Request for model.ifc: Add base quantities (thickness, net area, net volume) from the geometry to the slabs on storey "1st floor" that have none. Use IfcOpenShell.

First a look at what the model holds.

```python
import ifcopenshell
import ifcopenshell.util.element
import ifcopenshell.util.unit

model = ifcopenshell.open("model.ifc")
print(model.schema)
for unit_type in ("LENGTHUNIT", "AREAUNIT", "VOLUMEUNIT"):
    print(unit_type, ifcopenshell.util.unit.calculate_unit_scale(model, unit_type))
storey = next(s for s in model.by_type("IfcBuildingStorey") if s.Name == "1st floor")
slabs = [e for e in ifcopenshell.util.element.get_decomposition(storey) if e.is_a("IfcSlab")]
for e in sorted(slabs, key=lambda e: e.id()):
    print(e.id(), e.is_a(), e.Name, list(ifcopenshell.util.element.get_psets(e, qtos_only=True)), sep=" | ")
```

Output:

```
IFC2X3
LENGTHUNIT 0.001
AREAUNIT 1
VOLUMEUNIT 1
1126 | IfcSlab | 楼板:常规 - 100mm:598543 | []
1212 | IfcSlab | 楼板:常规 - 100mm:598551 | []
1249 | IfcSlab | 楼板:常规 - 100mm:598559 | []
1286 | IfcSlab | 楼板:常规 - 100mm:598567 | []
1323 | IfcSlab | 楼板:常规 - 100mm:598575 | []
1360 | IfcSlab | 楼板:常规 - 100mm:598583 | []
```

```python
import ifcopenshell
import ifcopenshell.api.pset
import ifcopenshell.geom
import ifcopenshell.util.element
import ifcopenshell.util.shape
import ifcopenshell.util.unit

model = ifcopenshell.open("model.ifc")
unit_scale = ifcopenshell.util.unit.calculate_unit_scale(model)
area_scale = ifcopenshell.util.unit.calculate_unit_scale(model, "AREAUNIT")
volume_scale = ifcopenshell.util.unit.calculate_unit_scale(model, "VOLUMEUNIT")
settings = ifcopenshell.geom.settings()

storey = next(s for s in model.by_type("IfcBuildingStorey") if s.Name == "1st floor")
slabs = [e for e in ifcopenshell.util.element.get_decomposition(storey) if e.is_a("IfcSlab")]

for e in sorted(slabs, key=lambda e: e.id()):
    if ifcopenshell.util.element.get_psets(e, qtos_only=True, should_inherit=False):
        continue
    # Geometry comes back in metres, in the element's own axes.
    shape = ifcopenshell.geom.create_shape(settings, e)
    values = {
        "Width": ifcopenshell.util.shape.get_z(shape.geometry) / unit_scale,
        "NetArea": ifcopenshell.util.shape.get_footprint_area(shape.geometry) / area_scale,
        "NetVolume": ifcopenshell.util.shape.get_volume(shape.geometry) / volume_scale,
    }
    qto = ifcopenshell.api.pset.add_qto(model, product=e, name="BaseQuantities")
    ifcopenshell.api.pset.edit_qto(model, qto=qto, properties=values)
    print(e.id(), {k: round(v, 3) for k, v in values.items()})

model.write("model_updated.ifc")
```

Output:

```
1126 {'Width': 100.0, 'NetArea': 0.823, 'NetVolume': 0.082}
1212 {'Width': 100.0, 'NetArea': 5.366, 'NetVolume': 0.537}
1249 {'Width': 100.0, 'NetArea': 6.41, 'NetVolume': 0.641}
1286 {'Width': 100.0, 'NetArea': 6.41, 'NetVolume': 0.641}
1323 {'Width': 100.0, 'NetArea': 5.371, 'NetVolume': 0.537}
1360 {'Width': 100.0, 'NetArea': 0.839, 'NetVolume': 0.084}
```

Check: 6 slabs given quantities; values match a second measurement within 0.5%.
